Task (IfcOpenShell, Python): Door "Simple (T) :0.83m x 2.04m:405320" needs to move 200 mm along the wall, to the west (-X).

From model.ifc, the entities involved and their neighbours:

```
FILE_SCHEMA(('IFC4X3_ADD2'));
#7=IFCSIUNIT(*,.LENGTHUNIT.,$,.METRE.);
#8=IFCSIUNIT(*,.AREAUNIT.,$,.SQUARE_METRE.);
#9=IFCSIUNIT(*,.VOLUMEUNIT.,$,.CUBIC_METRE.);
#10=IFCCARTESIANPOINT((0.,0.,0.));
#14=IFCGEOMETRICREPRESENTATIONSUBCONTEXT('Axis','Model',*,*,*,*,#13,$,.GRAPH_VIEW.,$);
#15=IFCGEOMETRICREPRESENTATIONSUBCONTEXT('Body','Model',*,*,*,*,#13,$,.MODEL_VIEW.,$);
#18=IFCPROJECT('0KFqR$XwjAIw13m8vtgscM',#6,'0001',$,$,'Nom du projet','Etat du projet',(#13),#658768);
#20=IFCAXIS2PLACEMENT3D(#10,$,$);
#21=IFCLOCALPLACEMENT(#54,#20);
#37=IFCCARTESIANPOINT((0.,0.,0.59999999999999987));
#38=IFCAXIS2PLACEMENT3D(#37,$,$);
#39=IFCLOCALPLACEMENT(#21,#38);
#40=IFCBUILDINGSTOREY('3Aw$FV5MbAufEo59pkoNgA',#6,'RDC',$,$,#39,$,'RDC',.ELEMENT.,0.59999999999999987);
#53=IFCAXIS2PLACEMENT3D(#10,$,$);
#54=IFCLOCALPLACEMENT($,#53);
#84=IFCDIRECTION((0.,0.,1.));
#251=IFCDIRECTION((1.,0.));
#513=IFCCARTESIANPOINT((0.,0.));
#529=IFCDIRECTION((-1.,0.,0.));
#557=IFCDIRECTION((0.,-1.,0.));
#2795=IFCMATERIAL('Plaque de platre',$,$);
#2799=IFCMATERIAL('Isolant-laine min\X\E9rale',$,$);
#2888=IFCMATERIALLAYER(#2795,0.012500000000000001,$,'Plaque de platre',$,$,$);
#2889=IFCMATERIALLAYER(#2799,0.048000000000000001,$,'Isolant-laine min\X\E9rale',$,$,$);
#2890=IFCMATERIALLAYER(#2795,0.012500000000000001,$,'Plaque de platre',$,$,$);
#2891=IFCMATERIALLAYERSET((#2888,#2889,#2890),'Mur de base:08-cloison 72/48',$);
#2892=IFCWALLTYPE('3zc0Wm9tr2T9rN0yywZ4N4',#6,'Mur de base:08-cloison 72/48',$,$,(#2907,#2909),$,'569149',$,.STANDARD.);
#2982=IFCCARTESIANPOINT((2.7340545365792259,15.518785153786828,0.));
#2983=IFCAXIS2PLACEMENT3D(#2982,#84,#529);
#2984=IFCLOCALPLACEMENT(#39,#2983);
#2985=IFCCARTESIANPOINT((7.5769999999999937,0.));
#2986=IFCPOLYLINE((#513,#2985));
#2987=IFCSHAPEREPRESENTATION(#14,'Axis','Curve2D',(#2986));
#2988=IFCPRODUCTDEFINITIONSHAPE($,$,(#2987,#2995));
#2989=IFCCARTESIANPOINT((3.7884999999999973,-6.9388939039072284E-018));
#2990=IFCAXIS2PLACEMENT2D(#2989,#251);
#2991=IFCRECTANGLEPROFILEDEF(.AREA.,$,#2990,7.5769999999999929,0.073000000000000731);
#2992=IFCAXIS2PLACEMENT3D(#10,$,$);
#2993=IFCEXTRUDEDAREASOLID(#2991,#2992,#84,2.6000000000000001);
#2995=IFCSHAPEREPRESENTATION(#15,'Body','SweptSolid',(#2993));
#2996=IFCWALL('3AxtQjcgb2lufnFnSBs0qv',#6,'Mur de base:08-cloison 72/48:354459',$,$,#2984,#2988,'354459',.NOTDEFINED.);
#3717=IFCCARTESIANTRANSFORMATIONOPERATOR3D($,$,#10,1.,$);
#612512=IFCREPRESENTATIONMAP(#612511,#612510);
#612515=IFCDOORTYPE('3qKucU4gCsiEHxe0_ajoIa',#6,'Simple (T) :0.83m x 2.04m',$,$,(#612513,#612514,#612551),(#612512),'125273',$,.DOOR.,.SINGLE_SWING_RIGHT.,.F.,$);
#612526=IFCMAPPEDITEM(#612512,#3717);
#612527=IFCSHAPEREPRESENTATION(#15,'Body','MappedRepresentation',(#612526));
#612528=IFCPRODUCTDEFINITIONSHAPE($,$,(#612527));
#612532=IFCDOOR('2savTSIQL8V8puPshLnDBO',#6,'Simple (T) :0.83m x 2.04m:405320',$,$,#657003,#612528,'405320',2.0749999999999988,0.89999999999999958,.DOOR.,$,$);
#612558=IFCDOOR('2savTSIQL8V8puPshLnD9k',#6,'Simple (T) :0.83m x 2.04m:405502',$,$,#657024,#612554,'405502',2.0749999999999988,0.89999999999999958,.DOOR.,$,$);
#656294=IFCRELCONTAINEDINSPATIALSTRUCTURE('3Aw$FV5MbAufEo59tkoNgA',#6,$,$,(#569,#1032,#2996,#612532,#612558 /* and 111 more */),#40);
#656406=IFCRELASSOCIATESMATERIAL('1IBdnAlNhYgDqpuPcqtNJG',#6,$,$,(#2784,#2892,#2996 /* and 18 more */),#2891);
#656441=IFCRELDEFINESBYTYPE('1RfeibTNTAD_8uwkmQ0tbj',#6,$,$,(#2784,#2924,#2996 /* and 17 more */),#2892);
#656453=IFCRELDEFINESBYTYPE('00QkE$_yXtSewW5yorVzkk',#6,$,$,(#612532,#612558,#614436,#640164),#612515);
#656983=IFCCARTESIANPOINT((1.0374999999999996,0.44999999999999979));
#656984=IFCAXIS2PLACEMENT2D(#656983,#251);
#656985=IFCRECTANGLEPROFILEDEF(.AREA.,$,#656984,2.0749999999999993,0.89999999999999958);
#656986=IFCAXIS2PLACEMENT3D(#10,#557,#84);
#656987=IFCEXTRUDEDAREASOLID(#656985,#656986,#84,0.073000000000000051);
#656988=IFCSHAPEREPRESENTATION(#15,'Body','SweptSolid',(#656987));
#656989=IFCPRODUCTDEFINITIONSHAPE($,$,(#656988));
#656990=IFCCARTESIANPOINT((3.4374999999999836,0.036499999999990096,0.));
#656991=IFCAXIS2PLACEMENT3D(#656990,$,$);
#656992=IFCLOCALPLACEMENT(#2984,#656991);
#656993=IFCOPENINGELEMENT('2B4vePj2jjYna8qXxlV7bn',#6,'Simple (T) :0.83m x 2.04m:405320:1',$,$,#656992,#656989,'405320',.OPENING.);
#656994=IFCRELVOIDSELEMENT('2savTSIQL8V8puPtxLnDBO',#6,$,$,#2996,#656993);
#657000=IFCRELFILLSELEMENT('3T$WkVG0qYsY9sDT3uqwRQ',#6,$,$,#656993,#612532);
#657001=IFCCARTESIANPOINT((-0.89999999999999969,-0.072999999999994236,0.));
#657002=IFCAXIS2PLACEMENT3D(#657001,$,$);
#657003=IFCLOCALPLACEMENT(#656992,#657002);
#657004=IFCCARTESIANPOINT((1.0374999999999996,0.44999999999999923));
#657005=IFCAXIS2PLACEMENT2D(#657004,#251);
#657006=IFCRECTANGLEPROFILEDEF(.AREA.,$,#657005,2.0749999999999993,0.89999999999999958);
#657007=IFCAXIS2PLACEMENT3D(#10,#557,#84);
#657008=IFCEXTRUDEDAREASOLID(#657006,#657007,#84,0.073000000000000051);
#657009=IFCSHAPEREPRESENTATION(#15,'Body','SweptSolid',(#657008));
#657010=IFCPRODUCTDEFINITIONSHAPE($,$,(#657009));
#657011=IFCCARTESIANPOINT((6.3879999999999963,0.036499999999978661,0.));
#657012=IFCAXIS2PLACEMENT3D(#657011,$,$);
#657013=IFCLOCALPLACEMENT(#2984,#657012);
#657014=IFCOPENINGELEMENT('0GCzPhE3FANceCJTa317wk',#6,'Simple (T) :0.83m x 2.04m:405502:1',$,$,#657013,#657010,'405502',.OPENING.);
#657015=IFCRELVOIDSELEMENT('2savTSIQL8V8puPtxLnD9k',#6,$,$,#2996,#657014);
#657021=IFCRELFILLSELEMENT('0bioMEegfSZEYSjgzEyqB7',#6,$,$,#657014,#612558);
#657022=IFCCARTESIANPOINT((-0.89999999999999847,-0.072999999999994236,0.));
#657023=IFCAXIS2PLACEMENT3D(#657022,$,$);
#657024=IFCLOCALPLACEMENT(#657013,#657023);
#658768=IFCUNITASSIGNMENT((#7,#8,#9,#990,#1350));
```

```python
import ifcopenshell
import ifcopenshell.api.geometry
import ifcopenshell.util.placement
import ifcopenshell.util.unit

model = ifcopenshell.open("model.ifc")
unit_scale = ifcopenshell.util.unit.calculate_unit_scale(model)

door = model.by_guid("2savTSIQL8V8puPshLnDBO")
opening = door.FillsVoids[0].RelatingOpeningElement
wall = opening.VoidsElements[0].RelatingBuildingElement

wall_matrix = ifcopenshell.util.placement.get_local_placement(wall.ObjectPlacement)
shift = wall_matrix[:3, 0] * 0.2 / unit_scale
before = ifcopenshell.util.placement.get_local_placement(door.ObjectPlacement)[:3, 3].copy()

# The door is placed relative to its opening, so it follows when the opening moves.
matrix = ifcopenshell.util.placement.get_local_placement(opening.ObjectPlacement)
matrix[:3, 3] += shift
ifcopenshell.api.geometry.edit_object_placement(
    model, product=opening, matrix=matrix, is_si=False, should_transform_children=True
)

after = ifcopenshell.util.placement.get_local_placement(door.ObjectPlacement)[:3, 3]
print("door moved by", (after - before).round(3) + 0.0)

model.write("model_rev.ifc")
```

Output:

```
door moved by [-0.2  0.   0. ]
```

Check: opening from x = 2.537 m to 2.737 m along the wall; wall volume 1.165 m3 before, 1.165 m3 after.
